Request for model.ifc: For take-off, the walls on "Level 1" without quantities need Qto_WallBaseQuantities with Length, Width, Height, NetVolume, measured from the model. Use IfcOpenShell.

First a look at what the model holds.

```python
import ifcopenshell
import ifcopenshell.util.element
import ifcopenshell.util.unit

model = ifcopenshell.open("model.ifc")
print(model.schema)
for unit_type in ("LENGTHUNIT", "AREAUNIT", "VOLUMEUNIT"):
    print(unit_type, ifcopenshell.util.unit.calculate_unit_scale(model, unit_type))
storey = next(s for s in model.by_type("IfcBuildingStorey") if s.Name == "Level 1")
walls = [e for e in ifcopenshell.util.element.get_decomposition(storey) if e.is_a("IfcWall")]
for e in sorted(walls, key=lambda e: e.id()):
    print(e.id(), e.is_a(), e.Name, list(ifcopenshell.util.element.get_psets(e, qtos_only=True)), sep=" | ")
```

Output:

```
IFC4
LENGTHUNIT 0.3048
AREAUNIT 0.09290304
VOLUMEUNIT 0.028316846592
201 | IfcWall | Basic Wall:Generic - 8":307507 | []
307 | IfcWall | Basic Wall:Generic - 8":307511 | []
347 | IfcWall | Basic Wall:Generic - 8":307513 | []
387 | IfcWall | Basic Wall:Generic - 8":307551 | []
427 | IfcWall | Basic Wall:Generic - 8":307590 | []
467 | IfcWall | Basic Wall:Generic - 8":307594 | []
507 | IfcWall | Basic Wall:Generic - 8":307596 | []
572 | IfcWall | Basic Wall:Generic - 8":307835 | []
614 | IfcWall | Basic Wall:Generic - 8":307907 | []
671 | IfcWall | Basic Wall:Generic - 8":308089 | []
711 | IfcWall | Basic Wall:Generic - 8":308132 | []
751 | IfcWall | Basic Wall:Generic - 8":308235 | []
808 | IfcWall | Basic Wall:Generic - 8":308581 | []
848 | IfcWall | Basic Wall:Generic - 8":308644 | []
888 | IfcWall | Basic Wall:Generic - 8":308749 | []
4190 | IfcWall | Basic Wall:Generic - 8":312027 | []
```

```python
import ifcopenshell
import ifcopenshell.api.pset
import ifcopenshell.geom
import ifcopenshell.util.element
import ifcopenshell.util.shape
import ifcopenshell.util.unit

model = ifcopenshell.open("model.ifc")
unit_scale = ifcopenshell.util.unit.calculate_unit_scale(model)
volume_scale = ifcopenshell.util.unit.calculate_unit_scale(model, "VOLUMEUNIT")
settings = ifcopenshell.geom.settings()

storey = next(s for s in model.by_type("IfcBuildingStorey") if s.Name == "Level 1")
walls = [e for e in ifcopenshell.util.element.get_decomposition(storey) if e.is_a("IfcWall")]

for e in sorted(walls, key=lambda e: e.id()):
    if ifcopenshell.util.element.get_psets(e, qtos_only=True, should_inherit=False):
        continue
    # Geometry comes back in metres, in the element's own axes.
    shape = ifcopenshell.geom.create_shape(settings, e)
    values = {
        "Length": ifcopenshell.util.shape.get_x(shape.geometry) / unit_scale,
        "Width": ifcopenshell.util.shape.get_y(shape.geometry) / unit_scale,
        "Height": ifcopenshell.util.shape.get_z(shape.geometry) / unit_scale,
        "NetVolume": ifcopenshell.util.shape.get_volume(shape.geometry) / volume_scale,
    }
    qto = ifcopenshell.api.pset.add_qto(model, product=e, name="Qto_WallBaseQuantities")
    ifcopenshell.api.pset.edit_qto(model, qto=qto, properties=values)
    print(e.id(), {k: round(v, 3) for k, v in values.items()})

model.write("model_v2.ifc")
```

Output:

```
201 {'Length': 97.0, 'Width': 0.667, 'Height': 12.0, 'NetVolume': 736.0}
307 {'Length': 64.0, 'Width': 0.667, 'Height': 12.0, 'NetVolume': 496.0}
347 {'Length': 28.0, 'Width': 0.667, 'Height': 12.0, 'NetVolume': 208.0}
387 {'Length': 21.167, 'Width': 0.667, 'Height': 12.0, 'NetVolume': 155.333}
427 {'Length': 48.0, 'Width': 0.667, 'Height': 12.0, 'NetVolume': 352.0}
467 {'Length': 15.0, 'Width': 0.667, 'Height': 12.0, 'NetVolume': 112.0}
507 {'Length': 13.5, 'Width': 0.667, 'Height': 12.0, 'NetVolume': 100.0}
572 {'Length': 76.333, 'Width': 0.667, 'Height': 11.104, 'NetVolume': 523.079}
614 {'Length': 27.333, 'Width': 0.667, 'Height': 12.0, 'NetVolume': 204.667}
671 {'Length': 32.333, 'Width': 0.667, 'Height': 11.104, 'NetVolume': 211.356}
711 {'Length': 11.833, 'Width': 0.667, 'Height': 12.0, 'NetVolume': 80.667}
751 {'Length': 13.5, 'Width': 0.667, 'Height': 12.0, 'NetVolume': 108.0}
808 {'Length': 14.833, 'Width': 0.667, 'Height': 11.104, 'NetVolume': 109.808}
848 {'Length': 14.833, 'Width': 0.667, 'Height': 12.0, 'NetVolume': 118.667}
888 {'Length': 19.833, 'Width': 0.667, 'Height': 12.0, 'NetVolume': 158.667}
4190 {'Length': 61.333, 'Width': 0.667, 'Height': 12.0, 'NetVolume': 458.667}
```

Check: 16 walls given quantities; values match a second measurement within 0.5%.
